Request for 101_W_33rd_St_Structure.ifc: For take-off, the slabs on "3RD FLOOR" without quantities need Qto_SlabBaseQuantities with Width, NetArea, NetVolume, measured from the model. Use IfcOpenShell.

First a look at what the model holds.

```python
import ifcopenshell
import ifcopenshell.util.element
import ifcopenshell.util.unit

model = ifcopenshell.open("101_W_33rd_St_Structure.ifc")
print(model.schema)
for unit_type in ("LENGTHUNIT", "AREAUNIT", "VOLUMEUNIT"):
    print(unit_type, ifcopenshell.util.unit.calculate_unit_scale(model, unit_type))
storey = next(s for s in model.by_type("IfcBuildingStorey") if s.Name == "3RD FLOOR")
slabs = [e for e in ifcopenshell.util.element.get_decomposition(storey) if e.is_a("IfcSlab")]
for e in sorted(slabs, key=lambda e: e.id()):
    print(e.id(), e.is_a(), e.Name, list(ifcopenshell.util.element.get_psets(e, qtos_only=True)), sep=" | ")
```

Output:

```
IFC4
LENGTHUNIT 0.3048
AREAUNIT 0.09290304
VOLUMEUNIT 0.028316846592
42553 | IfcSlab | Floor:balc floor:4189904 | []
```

```python
import ifcopenshell
import ifcopenshell.api.pset
import ifcopenshell.geom
import ifcopenshell.util.element
import ifcopenshell.util.shape
import ifcopenshell.util.unit

model = ifcopenshell.open("101_W_33rd_St_Structure.ifc")
unit_scale = ifcopenshell.util.unit.calculate_unit_scale(model)
area_scale = ifcopenshell.util.unit.calculate_unit_scale(model, "AREAUNIT")
volume_scale = ifcopenshell.util.unit.calculate_unit_scale(model, "VOLUMEUNIT")
settings = ifcopenshell.geom.settings()

storey = next(s for s in model.by_type("IfcBuildingStorey") if s.Name == "3RD FLOOR")
slabs = [e for e in ifcopenshell.util.element.get_decomposition(storey) if e.is_a("IfcSlab")]

for e in sorted(slabs, key=lambda e: e.id()):
    if ifcopenshell.util.element.get_psets(e, qtos_only=True, should_inherit=False):
        continue
    # Geometry comes back in metres, in the element's own axes.
    shape = ifcopenshell.geom.create_shape(settings, e)
    values = {
        "Width": ifcopenshell.util.shape.get_z(shape.geometry) / unit_scale,
        "NetArea": ifcopenshell.util.shape.get_footprint_area(shape.geometry) / area_scale,
        "NetVolume": ifcopenshell.util.shape.get_volume(shape.geometry) / volume_scale,
    }
    qto = ifcopenshell.api.pset.add_qto(model, product=e, name="Qto_SlabBaseQuantities")
    ifcopenshell.api.pset.edit_qto(model, qto=qto, properties=values)
    print(e.id(), {k: round(v, 3) for k, v in values.items()})

model.write("101_W_33rd_St_Structure_edited.ifc")
```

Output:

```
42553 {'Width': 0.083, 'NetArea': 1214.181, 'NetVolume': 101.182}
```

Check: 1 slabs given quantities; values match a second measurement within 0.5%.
